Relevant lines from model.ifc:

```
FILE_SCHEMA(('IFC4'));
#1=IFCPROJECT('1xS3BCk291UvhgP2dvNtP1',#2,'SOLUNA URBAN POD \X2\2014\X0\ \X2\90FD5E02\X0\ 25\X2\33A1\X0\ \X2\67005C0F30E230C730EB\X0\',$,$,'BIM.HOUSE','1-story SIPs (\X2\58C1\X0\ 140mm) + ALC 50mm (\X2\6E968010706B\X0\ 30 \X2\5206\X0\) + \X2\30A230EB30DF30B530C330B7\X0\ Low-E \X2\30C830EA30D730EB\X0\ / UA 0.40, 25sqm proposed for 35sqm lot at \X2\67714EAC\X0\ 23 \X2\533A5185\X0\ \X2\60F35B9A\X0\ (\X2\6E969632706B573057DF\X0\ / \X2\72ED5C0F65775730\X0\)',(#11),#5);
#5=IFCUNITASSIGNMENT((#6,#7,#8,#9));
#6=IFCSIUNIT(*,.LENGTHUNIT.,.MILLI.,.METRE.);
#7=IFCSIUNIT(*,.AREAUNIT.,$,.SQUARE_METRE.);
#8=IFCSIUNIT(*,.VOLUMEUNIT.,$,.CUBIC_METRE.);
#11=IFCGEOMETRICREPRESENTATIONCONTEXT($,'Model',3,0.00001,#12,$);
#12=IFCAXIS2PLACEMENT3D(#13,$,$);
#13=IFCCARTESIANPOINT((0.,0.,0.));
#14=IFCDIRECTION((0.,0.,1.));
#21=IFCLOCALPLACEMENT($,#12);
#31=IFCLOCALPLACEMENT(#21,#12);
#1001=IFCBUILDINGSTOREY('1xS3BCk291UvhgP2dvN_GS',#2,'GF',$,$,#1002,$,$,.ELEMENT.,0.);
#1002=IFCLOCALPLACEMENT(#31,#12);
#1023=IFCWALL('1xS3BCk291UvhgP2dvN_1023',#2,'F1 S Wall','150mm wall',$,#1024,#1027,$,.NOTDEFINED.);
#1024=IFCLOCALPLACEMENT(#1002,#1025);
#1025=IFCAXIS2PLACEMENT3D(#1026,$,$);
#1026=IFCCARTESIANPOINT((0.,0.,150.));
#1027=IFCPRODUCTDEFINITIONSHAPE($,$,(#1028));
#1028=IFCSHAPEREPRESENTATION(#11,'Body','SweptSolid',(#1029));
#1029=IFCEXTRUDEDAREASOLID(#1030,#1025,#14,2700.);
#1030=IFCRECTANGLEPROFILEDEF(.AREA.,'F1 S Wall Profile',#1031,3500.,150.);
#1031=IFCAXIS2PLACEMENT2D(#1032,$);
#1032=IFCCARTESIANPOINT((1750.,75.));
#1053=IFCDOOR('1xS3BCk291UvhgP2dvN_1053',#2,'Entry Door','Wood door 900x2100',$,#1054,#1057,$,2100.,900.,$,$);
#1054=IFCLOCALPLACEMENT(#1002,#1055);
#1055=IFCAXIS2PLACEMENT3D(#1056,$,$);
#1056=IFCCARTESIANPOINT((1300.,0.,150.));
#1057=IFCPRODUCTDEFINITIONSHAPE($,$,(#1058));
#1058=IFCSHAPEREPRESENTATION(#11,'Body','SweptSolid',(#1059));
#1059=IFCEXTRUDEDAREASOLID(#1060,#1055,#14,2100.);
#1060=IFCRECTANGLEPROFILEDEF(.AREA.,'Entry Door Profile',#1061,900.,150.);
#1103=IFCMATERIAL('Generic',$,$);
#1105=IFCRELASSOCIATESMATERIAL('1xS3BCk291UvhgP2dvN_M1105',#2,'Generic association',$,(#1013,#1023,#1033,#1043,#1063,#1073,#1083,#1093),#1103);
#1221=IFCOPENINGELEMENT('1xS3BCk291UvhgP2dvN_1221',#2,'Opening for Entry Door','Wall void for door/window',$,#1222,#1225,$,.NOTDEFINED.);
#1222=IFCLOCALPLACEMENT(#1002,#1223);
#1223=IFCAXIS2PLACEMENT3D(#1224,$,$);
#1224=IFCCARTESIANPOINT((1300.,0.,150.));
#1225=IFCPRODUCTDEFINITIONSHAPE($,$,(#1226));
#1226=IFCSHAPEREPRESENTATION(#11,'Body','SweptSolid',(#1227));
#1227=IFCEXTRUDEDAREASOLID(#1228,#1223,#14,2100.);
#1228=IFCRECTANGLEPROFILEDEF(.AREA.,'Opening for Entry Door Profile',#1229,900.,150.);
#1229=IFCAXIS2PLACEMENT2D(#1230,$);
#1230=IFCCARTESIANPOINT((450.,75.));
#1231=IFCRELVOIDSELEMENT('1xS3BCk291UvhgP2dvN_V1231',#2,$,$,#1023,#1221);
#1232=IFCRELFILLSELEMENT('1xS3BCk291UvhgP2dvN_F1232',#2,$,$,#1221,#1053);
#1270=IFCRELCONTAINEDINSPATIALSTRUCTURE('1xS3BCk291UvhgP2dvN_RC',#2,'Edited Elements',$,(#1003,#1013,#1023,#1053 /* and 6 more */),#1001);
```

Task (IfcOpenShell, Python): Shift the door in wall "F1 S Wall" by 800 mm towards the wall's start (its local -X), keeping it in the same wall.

```python
import ifcopenshell
import ifcopenshell.api.geometry
import ifcopenshell.util.placement
import ifcopenshell.util.unit

model = ifcopenshell.open("model.ifc")
unit_scale = ifcopenshell.util.unit.calculate_unit_scale(model)

door = model.by_guid("1xS3BCk291UvhgP2dvN_1053")
opening = door.FillsVoids[0].RelatingOpeningElement
wall = opening.VoidsElements[0].RelatingBuildingElement

wall_matrix = ifcopenshell.util.placement.get_local_placement(wall.ObjectPlacement)
shift = wall_matrix[:3, 0] * -0.8 / unit_scale
before = ifcopenshell.util.placement.get_local_placement(door.ObjectPlacement)[:3, 3].copy()

# The door is not placed relative to its opening, so move both.
for product in (opening, door):
    matrix = ifcopenshell.util.placement.get_local_placement(product.ObjectPlacement)
    matrix[:3, 3] += shift
    ifcopenshell.api.geometry.edit_object_placement(model, product=product, matrix=matrix, is_si=False)

after = ifcopenshell.util.placement.get_local_placement(door.ObjectPlacement)[:3, 3]
print("door moved by", (after - before).round(3) + 0.0)

model.write("model_edited.ifc")
```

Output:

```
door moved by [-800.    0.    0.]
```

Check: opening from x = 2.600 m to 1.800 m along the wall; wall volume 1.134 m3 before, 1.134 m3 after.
